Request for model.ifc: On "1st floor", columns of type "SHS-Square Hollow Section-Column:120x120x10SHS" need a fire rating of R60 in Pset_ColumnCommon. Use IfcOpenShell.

First a look at what the model holds.

```python
import ifcopenshell
import ifcopenshell.util.element

model = ifcopenshell.open("model.ifc")
print(model.schema)
storey = next(s for s in model.by_type("IfcBuildingStorey") if s.Name == "1st floor")
columns = [e for e in ifcopenshell.util.element.get_decomposition(storey) if e.is_a("IfcColumn")]
seen = {}
for e in columns:
    element_type = ifcopenshell.util.element.get_type(e)
    key = (element_type.Name if element_type != e and element_type else None, ifcopenshell.util.element.get_pset(e, "Pset_ColumnCommon", "FireRating"))
    seen[key] = seen.get(key, 0) + 1
for (name, value), count in sorted(seen.items(), key=str):
    print(count, "x", name, "|", value)
```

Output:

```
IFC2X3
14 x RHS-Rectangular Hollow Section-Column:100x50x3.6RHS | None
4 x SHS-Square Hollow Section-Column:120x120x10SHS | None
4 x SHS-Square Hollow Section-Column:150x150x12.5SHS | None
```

```python
import ifcopenshell
import ifcopenshell.api.pset
import ifcopenshell.util.element

model = ifcopenshell.open("model.ifc")

storey = next(s for s in model.by_type("IfcBuildingStorey") if s.Name == "1st floor")
columns = [e for e in ifcopenshell.util.element.get_decomposition(storey) if e.is_a("IfcColumn")]

count = 0
for e in columns:
    element_type = ifcopenshell.util.element.get_type(e)
    if element_type in (None, e) or element_type.Name != "SHS-Square Hollow Section-Column:120x120x10SHS":
        continue
    # add_pset returns the element's existing set when there is one.
    pset = ifcopenshell.api.pset.add_pset(model, product=e, name="Pset_ColumnCommon")
    ifcopenshell.api.pset.edit_pset(model, pset=pset, properties={"FireRating": "R60"})
    count += 1

print(count, "columns updated")

model.write("model_rev.ifc")
```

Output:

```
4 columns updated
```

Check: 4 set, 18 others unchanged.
